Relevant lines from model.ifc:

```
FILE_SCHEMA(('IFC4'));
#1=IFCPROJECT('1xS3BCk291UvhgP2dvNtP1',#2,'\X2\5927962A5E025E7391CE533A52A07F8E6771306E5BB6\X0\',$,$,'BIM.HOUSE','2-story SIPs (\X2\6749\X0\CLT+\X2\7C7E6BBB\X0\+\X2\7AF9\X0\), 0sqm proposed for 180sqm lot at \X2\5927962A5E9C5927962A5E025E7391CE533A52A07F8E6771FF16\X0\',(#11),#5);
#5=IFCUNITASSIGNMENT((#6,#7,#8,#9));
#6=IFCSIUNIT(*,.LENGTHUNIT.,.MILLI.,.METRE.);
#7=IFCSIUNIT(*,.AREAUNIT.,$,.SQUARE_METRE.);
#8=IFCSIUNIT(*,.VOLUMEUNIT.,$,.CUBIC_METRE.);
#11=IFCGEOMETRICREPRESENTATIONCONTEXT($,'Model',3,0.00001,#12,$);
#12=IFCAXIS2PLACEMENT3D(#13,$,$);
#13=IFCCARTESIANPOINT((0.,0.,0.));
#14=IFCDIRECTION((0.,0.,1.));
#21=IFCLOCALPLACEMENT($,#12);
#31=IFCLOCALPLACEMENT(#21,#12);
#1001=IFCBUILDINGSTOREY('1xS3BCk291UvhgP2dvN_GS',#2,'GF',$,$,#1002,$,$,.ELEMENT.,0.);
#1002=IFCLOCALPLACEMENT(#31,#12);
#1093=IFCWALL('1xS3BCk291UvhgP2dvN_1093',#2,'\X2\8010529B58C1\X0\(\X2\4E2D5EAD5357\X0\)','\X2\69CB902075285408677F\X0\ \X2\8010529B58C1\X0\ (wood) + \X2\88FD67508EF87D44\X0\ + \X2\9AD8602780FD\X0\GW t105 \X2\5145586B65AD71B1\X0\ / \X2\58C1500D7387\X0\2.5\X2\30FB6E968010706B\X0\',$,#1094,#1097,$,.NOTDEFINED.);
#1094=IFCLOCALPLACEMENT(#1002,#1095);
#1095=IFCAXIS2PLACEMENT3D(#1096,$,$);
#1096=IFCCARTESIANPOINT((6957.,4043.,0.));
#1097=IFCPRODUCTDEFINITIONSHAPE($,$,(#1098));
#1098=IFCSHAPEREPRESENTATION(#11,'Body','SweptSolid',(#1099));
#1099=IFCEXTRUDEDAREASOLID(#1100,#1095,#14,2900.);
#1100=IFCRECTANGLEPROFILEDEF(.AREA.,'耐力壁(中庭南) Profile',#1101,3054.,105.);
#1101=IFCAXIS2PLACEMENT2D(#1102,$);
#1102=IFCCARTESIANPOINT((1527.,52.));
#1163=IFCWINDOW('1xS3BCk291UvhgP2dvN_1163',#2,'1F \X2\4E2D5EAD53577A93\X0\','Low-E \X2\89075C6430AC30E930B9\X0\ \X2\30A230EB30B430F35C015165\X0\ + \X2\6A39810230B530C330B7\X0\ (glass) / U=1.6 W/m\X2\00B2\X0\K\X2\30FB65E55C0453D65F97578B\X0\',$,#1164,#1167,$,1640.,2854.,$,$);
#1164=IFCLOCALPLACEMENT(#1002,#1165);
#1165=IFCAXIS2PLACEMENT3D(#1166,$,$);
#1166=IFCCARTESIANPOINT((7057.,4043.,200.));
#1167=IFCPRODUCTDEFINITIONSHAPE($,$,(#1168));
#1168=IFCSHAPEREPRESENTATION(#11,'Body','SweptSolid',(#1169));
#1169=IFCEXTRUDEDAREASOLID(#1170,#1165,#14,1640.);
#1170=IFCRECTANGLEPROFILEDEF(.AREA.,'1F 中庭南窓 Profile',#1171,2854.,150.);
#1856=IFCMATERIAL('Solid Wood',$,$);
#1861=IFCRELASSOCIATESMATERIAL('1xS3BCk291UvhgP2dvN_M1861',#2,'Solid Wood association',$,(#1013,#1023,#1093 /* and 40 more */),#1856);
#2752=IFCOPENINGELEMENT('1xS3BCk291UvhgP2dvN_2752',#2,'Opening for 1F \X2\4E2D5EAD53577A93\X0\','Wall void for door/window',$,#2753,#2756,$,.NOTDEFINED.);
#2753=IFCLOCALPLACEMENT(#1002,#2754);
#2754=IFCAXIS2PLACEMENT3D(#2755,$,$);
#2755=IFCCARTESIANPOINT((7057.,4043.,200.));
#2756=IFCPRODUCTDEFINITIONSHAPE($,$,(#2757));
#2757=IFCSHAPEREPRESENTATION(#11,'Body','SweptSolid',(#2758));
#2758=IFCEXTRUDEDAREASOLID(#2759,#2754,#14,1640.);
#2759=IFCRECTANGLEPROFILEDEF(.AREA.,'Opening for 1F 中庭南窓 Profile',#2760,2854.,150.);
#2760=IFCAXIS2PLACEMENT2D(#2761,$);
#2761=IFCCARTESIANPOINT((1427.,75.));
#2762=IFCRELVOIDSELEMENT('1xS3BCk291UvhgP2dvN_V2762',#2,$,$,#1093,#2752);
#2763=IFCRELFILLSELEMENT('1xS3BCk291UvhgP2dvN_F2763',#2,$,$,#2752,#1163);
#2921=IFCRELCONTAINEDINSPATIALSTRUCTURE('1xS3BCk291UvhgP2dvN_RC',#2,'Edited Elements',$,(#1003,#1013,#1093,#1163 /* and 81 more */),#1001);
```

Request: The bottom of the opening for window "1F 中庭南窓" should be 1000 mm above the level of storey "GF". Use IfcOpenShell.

```python
import numpy as np
import ifcopenshell
import ifcopenshell.api.geometry
import ifcopenshell.geom
import ifcopenshell.util.element
import ifcopenshell.util.placement
import ifcopenshell.util.shape
import ifcopenshell.util.unit

model = ifcopenshell.open("model.ifc")
unit_scale = ifcopenshell.util.unit.calculate_unit_scale(model)

window = model.by_guid("1xS3BCk291UvhgP2dvN_1163")
opening = window.FillsVoids[0].RelatingOpeningElement
storey = ifcopenshell.util.element.get_container(window, ifc_class="IfcBuildingStorey")
level = ifcopenshell.util.placement.get_local_placement(storey.ObjectPlacement)[2, 3]

# The opening's origin need not be at the sill, so measure its lowest point.
shape = ifcopenshell.geom.create_shape(ifcopenshell.geom.settings(), opening)
bottom = ifcopenshell.util.shape.get_shape_bottom_elevation(shape, shape.geometry) / unit_scale
dz = level + 1 / unit_scale - bottom

shift = np.array([0.0, 0.0, dz])
# The window is not placed relative to its opening, so move both.
for product in (opening, window):
    matrix = ifcopenshell.util.placement.get_local_placement(product.ObjectPlacement)
    matrix[:3, 3] += shift
    ifcopenshell.api.geometry.edit_object_placement(model, product=product, matrix=matrix, is_si=False)

print(f"moved by {dz * unit_scale:+.3f} m")

model.write("model_edited.ifc")
```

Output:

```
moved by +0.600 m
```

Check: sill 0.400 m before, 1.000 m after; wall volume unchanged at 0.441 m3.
